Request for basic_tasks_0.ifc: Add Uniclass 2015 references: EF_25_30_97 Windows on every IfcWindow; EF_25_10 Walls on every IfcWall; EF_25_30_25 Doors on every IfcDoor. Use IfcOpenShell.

First a look at what the model holds.

```python
import ifcopenshell

model = ifcopenshell.open("basic_tasks_0.ifc")
print(model.schema)
print("classifications:", [c.Name for c in model.by_type("IfcClassification")])
for ifc_class in ("IfcDoor", "IfcRoof", "IfcStair", "IfcWall", "IfcWindow"):
    print(ifc_class, len(model.by_type(ifc_class)))
```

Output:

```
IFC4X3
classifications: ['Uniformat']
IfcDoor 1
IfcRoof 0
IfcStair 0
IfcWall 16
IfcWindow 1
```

```python
import ifcopenshell
import ifcopenshell.api.classification

model = ifcopenshell.open("basic_tasks_0.ifc")

system = ifcopenshell.api.classification.add_classification(model, classification="Uniclass 2015")

codes = {
    "IfcWindow": ("EF_25_30_97", "Windows"),
    "IfcWall": ("EF_25_10", "Walls"),
    "IfcDoor": ("EF_25_30_25", "Doors"),
}
for ifc_class, (code, name) in codes.items():
    products = model.by_type(ifc_class)
    ifcopenshell.api.classification.add_reference(
        model, products=products, classification=system, identification=code, name=name
    )
    print(code, len(products))

model.write("basic_tasks_0_edited.ifc")
```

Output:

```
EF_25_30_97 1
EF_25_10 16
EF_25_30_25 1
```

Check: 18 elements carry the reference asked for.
